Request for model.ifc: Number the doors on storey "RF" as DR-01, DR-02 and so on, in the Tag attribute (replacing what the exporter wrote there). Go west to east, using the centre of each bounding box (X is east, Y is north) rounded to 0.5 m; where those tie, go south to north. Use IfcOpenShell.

First a look at what the model holds.

```python
import ifcopenshell
import ifcopenshell.util.element
import ifcopenshell.util.placement

model = ifcopenshell.open("model.ifc")
print(model.schema)
storey = next(s for s in model.by_type("IfcBuildingStorey") if s.Name == "RF")
doors = [e for e in ifcopenshell.util.element.get_decomposition(storey) if e.is_a("IfcDoor")]
for e in sorted(doors, key=lambda e: e.id()):
    origin = ifcopenshell.util.placement.get_local_placement(e.ObjectPlacement)[:3, 3]
    print(e.id(), e.Tag, e.Name, origin.round(2) + 0.0, sep=" | ")
```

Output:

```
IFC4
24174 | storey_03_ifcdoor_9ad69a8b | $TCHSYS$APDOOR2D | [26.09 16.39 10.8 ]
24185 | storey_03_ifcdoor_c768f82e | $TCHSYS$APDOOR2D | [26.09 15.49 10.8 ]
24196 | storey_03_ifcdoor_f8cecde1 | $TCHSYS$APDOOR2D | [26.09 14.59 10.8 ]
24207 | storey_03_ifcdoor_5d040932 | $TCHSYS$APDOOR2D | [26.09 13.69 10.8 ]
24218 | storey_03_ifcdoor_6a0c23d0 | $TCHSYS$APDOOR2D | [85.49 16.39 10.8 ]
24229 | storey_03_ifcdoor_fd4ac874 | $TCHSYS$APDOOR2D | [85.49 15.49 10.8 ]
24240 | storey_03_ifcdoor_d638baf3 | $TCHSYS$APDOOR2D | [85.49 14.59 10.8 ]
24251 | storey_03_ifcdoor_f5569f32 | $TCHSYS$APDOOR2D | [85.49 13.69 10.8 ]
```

```python
import ifcopenshell
import ifcopenshell.geom
import ifcopenshell.util.element
import ifcopenshell.util.shape

model = ifcopenshell.open("model.ifc")
settings = ifcopenshell.geom.settings()
settings.set("use-world-coords", True)


def centre(element):
    shape = ifcopenshell.geom.create_shape(settings, element)
    return ifcopenshell.util.shape.get_bbox_centroid(shape.geometry)


storey = next(s for s in model.by_type("IfcBuildingStorey") if s.Name == "RF")
doors = [e for e in ifcopenshell.util.element.get_decomposition(storey) if e.is_a("IfcDoor")]

# Insertion points can sit at a corner or the storey origin, so sort by the geometry (in metres).
centres = {e: centre(e) for e in doors}
doors.sort(key=lambda e: (round(centres[e][0] / 0.5), centres[e][1]))

for i, e in enumerate(doors, start=1):
    number = f"DR-{i:02d}"
    e.Tag = number
    print(e.id(), number)

model.write("model_v2.ifc")
```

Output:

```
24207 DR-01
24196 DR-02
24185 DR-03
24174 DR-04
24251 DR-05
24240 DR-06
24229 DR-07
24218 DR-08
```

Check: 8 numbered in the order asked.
